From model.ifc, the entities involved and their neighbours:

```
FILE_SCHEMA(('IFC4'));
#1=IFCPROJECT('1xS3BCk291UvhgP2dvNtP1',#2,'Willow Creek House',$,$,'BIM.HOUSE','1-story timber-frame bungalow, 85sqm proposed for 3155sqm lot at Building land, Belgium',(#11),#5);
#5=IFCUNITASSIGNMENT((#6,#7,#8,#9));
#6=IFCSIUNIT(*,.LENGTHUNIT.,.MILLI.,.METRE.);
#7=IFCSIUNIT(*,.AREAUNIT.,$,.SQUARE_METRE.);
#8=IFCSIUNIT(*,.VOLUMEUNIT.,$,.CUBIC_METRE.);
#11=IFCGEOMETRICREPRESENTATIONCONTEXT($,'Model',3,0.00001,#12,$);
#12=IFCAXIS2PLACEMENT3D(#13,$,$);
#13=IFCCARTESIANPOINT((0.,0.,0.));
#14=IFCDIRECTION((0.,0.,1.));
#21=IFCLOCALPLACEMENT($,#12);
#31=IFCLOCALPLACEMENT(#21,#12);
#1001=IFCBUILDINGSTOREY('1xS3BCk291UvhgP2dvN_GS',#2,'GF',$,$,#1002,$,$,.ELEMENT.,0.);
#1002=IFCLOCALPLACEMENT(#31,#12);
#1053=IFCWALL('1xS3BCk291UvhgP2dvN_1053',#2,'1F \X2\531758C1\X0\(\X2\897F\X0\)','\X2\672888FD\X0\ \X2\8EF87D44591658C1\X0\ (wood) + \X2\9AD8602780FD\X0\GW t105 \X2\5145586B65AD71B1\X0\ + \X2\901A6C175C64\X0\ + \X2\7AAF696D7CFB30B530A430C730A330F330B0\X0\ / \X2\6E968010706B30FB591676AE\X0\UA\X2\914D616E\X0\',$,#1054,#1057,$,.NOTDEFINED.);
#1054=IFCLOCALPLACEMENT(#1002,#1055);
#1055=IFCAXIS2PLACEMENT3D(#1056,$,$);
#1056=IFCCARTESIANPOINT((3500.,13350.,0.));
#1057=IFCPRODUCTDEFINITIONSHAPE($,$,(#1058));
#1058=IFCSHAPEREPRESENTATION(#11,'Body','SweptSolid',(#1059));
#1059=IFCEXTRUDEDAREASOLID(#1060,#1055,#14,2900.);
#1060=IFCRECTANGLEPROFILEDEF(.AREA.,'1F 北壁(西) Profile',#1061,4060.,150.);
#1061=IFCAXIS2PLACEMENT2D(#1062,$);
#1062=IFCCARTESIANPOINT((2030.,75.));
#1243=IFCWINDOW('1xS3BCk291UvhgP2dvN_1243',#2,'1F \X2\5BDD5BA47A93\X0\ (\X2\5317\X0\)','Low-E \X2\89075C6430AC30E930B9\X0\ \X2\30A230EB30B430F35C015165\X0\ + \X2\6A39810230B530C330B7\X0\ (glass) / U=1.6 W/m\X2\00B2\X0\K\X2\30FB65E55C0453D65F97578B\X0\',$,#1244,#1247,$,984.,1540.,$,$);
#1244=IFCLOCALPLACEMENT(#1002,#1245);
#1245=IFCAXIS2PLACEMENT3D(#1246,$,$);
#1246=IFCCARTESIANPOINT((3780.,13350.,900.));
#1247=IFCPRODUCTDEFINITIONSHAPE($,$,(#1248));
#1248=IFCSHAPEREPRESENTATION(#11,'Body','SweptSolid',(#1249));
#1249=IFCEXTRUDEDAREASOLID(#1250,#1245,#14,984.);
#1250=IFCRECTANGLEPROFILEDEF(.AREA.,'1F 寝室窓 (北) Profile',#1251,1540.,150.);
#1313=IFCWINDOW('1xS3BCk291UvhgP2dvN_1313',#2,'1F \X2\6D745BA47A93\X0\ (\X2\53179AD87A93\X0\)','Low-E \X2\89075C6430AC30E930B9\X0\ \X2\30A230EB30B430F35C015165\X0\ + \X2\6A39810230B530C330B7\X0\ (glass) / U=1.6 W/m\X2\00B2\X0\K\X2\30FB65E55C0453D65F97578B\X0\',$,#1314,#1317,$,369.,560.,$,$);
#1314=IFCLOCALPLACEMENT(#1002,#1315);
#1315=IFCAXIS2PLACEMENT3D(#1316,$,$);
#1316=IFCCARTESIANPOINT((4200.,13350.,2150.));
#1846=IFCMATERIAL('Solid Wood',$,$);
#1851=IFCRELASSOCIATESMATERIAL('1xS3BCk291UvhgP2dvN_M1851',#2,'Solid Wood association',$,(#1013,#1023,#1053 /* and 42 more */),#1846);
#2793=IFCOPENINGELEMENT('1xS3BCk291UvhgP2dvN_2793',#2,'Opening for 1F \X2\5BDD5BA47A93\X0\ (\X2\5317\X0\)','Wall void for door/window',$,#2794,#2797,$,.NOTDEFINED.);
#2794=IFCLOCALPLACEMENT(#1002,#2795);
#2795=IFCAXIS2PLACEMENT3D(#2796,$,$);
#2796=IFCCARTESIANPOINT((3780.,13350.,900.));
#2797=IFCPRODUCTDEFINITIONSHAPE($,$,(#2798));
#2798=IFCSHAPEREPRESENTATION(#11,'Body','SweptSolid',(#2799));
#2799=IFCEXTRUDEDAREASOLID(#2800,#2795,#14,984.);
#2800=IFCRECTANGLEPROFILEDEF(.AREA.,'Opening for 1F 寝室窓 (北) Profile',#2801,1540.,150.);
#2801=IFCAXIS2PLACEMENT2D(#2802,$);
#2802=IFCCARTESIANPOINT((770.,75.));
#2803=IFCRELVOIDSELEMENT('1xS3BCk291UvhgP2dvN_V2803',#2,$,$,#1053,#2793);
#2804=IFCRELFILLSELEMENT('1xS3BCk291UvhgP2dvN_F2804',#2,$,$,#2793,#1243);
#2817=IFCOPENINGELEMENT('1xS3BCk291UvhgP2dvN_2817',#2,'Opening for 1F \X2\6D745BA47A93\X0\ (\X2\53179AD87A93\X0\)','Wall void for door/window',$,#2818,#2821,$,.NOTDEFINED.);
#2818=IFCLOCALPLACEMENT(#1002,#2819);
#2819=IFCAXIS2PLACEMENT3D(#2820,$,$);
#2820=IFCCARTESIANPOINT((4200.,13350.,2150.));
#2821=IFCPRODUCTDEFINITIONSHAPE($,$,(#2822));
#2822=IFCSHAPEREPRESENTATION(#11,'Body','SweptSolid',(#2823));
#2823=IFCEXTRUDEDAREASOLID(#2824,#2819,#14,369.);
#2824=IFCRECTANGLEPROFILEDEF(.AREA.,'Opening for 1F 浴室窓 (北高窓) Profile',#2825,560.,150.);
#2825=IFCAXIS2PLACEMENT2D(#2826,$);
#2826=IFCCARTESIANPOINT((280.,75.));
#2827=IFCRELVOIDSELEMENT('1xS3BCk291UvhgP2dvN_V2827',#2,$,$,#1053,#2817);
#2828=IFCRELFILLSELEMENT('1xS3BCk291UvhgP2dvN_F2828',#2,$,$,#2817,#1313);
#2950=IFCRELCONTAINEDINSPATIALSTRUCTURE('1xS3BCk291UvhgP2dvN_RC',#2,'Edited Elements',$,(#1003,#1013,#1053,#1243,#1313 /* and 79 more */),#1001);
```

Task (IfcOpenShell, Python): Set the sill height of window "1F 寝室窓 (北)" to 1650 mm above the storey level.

```python
import numpy as np
import ifcopenshell
import ifcopenshell.api.geometry
import ifcopenshell.geom
import ifcopenshell.util.element
import ifcopenshell.util.placement
import ifcopenshell.util.shape
import ifcopenshell.util.unit

model = ifcopenshell.open("model.ifc")
unit_scale = ifcopenshell.util.unit.calculate_unit_scale(model)

window = model.by_id(1243)
opening = window.FillsVoids[0].RelatingOpeningElement
storey = ifcopenshell.util.element.get_container(window, ifc_class="IfcBuildingStorey")
level = ifcopenshell.util.placement.get_local_placement(storey.ObjectPlacement)[2, 3]

# The opening's origin need not be at the sill, so measure its lowest point.
shape = ifcopenshell.geom.create_shape(ifcopenshell.geom.settings(), opening)
bottom = ifcopenshell.util.shape.get_shape_bottom_elevation(shape, shape.geometry) / unit_scale
dz = level + 1650.0 - bottom

shift = np.array([0.0, 0.0, dz])
# The window is not placed relative to its opening, so move both.
for product in (opening, window):
    matrix = ifcopenshell.util.placement.get_local_placement(product.ObjectPlacement)
    matrix[:3, 3] += shift
    ifcopenshell.api.geometry.edit_object_placement(model, product=product, matrix=matrix, is_si=False)

print(f"moved by {dz * unit_scale:+.3f} m")

model.write("model_v2.ifc")
```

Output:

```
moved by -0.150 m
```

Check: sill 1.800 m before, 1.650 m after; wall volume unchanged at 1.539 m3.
